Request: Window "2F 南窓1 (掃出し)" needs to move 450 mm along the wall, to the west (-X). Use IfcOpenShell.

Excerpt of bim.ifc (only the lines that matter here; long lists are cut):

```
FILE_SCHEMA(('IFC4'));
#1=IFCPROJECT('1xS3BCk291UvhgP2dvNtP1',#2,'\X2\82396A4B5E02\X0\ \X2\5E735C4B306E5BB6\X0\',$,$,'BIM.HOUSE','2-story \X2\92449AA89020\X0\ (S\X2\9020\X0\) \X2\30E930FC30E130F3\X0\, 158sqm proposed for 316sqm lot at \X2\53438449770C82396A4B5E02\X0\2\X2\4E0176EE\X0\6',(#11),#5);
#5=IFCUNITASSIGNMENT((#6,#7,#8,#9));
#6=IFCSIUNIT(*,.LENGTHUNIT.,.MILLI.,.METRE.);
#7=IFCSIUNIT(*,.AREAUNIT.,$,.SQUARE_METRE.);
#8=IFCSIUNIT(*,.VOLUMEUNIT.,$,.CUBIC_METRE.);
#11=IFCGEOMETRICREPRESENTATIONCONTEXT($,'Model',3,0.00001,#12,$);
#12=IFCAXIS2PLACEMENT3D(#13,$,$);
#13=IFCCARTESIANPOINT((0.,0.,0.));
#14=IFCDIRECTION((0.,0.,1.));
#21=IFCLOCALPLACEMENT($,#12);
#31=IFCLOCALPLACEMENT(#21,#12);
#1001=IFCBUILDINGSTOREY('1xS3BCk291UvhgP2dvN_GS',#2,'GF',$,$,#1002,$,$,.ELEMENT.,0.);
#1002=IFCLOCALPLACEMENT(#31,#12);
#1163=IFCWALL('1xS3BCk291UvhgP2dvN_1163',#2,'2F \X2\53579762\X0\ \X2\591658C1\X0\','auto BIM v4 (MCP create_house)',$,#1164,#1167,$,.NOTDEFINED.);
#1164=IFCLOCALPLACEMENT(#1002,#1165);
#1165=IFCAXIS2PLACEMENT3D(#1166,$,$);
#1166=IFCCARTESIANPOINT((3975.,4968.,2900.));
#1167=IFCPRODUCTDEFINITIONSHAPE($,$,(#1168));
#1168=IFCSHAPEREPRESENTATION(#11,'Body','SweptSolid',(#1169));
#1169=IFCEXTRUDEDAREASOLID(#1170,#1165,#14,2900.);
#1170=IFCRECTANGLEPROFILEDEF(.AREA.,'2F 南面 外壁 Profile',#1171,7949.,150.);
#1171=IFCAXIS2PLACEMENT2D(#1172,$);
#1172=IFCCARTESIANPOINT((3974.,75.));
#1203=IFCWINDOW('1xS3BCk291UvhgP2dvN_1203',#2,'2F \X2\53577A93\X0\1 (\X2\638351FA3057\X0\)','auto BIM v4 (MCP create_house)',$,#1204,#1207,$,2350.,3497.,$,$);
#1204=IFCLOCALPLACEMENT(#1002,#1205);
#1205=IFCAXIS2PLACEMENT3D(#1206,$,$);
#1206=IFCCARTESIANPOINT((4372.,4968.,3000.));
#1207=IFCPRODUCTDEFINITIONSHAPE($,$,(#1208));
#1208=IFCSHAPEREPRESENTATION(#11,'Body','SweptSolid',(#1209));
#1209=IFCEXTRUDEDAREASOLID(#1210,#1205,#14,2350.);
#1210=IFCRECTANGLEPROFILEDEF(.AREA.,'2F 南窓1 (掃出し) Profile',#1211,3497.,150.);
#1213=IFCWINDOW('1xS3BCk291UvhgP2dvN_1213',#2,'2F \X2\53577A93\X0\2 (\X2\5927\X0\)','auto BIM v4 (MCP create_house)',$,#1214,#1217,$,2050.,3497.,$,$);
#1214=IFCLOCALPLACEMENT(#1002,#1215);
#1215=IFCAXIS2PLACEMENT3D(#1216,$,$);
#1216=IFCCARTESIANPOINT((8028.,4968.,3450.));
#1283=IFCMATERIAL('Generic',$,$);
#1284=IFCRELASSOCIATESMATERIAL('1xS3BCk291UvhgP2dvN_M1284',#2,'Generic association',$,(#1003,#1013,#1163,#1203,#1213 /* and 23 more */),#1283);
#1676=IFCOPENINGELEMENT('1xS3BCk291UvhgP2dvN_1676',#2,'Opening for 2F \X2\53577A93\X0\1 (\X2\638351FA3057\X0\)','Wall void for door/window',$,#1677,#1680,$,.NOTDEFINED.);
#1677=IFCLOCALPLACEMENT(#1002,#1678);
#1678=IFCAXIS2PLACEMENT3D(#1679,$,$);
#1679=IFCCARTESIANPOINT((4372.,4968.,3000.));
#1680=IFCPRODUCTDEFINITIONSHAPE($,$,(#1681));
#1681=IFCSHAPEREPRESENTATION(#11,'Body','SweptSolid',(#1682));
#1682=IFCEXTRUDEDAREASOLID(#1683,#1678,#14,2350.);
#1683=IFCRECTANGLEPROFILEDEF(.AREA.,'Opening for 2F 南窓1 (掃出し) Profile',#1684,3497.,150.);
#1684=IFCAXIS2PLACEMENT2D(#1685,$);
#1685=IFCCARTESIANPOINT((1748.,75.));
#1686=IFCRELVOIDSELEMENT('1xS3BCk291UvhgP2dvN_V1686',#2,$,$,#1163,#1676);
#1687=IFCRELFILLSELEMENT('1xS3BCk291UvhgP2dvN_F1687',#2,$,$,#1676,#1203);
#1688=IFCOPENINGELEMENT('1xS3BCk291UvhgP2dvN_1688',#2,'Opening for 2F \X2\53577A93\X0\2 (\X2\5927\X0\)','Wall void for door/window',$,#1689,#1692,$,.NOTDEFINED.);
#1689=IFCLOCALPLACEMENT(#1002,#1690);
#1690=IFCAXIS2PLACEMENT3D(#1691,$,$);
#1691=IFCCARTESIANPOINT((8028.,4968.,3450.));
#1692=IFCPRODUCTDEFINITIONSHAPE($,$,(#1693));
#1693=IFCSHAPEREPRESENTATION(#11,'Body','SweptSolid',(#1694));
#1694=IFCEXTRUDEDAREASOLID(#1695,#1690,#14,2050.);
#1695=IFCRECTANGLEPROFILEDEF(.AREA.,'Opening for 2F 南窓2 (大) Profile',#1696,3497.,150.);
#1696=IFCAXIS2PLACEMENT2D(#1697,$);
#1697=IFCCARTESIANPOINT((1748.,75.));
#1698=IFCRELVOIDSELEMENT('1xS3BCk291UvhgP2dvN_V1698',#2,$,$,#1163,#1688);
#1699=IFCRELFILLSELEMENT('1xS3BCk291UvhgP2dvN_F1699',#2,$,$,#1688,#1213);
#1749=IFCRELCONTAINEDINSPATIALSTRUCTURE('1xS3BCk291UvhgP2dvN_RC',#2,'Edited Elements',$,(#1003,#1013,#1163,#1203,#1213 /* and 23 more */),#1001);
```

```python
import ifcopenshell
import ifcopenshell.api.geometry
import ifcopenshell.util.placement

model = ifcopenshell.open("bim.ifc")

window = model.by_id(1203)
opening = window.FillsVoids[0].RelatingOpeningElement
wall = opening.VoidsElements[0].RelatingBuildingElement

wall_matrix = ifcopenshell.util.placement.get_local_placement(wall.ObjectPlacement)
shift = wall_matrix[:3, 0] * -450.0
before = ifcopenshell.util.placement.get_local_placement(window.ObjectPlacement)[:3, 3].copy()

# The window is not placed relative to its opening, so move both.
for product in (opening, window):
    matrix = ifcopenshell.util.placement.get_local_placement(product.ObjectPlacement)
    matrix[:3, 3] += shift
    ifcopenshell.api.geometry.edit_object_placement(model, product=product, matrix=matrix, is_si=False)

after = ifcopenshell.util.placement.get_local_placement(window.ObjectPlacement)[:3, 3]
print("window moved by", (after - before).round(3) + 0.0)

model.write("bim-out.ifc")
```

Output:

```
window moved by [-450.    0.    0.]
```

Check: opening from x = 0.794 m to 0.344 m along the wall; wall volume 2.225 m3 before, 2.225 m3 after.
